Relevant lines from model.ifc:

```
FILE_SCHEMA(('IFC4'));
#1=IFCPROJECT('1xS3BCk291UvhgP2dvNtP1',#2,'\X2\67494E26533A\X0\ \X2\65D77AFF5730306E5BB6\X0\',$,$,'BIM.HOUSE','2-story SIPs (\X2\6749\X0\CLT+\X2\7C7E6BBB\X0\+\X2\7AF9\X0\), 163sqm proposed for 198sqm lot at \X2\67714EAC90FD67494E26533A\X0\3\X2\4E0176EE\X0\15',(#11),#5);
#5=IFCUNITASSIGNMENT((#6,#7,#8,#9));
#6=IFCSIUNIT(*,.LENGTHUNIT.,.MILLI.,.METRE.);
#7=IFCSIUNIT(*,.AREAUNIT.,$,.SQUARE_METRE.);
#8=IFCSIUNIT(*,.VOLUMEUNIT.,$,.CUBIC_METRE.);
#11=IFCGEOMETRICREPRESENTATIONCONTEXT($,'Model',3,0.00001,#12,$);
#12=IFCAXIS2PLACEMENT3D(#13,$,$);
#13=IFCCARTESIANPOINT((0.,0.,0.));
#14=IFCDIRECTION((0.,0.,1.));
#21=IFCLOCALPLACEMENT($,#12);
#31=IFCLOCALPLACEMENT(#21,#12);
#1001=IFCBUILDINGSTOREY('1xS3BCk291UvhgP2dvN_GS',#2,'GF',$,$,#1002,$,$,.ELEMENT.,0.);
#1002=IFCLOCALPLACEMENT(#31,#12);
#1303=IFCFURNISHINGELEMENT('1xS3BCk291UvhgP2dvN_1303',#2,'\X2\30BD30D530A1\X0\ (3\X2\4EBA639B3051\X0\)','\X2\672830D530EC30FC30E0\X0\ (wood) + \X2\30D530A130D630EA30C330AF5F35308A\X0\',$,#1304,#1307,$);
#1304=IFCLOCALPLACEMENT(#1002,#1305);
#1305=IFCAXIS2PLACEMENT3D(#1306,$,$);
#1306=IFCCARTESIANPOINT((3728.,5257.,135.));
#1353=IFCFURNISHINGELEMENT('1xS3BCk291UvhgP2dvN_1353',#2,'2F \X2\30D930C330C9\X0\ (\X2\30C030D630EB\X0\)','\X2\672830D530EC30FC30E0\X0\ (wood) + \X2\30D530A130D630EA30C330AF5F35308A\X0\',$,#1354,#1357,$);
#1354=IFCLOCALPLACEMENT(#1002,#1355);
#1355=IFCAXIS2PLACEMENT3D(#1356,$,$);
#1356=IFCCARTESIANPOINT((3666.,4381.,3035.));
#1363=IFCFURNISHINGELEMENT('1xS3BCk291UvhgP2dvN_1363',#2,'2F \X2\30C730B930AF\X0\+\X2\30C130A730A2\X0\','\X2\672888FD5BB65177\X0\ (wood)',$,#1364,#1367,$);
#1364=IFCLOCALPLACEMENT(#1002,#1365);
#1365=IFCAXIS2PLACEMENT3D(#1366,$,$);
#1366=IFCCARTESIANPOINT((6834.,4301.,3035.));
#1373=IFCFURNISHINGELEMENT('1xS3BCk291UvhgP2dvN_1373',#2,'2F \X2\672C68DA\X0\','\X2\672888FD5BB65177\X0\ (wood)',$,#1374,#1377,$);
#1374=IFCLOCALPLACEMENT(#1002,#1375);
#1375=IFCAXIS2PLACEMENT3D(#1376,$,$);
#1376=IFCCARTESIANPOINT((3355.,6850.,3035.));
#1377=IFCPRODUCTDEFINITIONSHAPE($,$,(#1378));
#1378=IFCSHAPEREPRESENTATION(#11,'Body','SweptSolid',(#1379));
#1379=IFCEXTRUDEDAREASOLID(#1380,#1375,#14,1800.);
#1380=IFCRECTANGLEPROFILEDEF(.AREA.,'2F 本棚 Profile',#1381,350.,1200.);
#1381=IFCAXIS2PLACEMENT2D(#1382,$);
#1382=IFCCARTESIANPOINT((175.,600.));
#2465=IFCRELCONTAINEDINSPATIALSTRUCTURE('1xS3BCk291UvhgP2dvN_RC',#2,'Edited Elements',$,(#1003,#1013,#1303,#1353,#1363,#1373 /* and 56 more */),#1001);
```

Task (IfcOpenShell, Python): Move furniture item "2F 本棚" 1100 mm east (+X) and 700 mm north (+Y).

```python
import ifcopenshell
import ifcopenshell.api.geometry
import ifcopenshell.util.placement
import ifcopenshell.util.unit

model = ifcopenshell.open("model.ifc")
unit_scale = ifcopenshell.util.unit.calculate_unit_scale(model)

item = model.by_guid("1xS3BCk291UvhgP2dvN_1373")
matrix = ifcopenshell.util.placement.get_local_placement(item.ObjectPlacement)
matrix[0, 3] += 1.1 / unit_scale
matrix[1, 3] += 0.7 / unit_scale
ifcopenshell.api.geometry.edit_object_placement(model, product=item, matrix=matrix, is_si=False)

print(ifcopenshell.util.placement.get_local_placement(item.ObjectPlacement).round(3) + 0.0)

model.write("model_edited.ifc")
```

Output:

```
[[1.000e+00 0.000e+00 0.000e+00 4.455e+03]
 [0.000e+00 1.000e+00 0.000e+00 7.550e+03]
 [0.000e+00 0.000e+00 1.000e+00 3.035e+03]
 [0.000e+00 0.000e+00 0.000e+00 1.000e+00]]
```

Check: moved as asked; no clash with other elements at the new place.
